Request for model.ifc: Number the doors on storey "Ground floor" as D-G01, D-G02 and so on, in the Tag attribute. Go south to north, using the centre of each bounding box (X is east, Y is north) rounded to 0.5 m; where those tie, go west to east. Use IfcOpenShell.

First a look at what the model holds.

```python
import ifcopenshell
import ifcopenshell.util.element
import ifcopenshell.util.placement

model = ifcopenshell.open("model.ifc")
print(model.schema)
storey = next(s for s in model.by_type("IfcBuildingStorey") if s.Name == "Ground floor")
doors = [e for e in ifcopenshell.util.element.get_decomposition(storey) if e.is_a("IfcDoor")]
for e in sorted(doors, key=lambda e: e.id()):
    origin = ifcopenshell.util.placement.get_local_placement(e.ObjectPlacement)[:3, 3]
    print(e.id(), e.Tag, e.Name, origin.round(2) + 0.0, sep=" | ")
```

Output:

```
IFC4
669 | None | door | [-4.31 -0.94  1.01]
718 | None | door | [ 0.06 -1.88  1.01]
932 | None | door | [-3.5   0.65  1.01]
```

```python
import ifcopenshell
import ifcopenshell.geom
import ifcopenshell.util.element
import ifcopenshell.util.shape

model = ifcopenshell.open("model.ifc")
settings = ifcopenshell.geom.settings()
settings.set("use-world-coords", True)


def centre(element):
    shape = ifcopenshell.geom.create_shape(settings, element)
    return ifcopenshell.util.shape.get_bbox_centroid(shape.geometry)


storey = next(s for s in model.by_type("IfcBuildingStorey") if s.Name == "Ground floor")
doors = [e for e in ifcopenshell.util.element.get_decomposition(storey) if e.is_a("IfcDoor")]

# Insertion points can sit at a corner or the storey origin, so sort by the geometry (in metres).
centres = {e: centre(e) for e in doors}
doors.sort(key=lambda e: (round(centres[e][1] / 0.5), centres[e][0]))

for i, e in enumerate(doors, start=1):
    number = f"D-G{i:02d}"
    e.Tag = number
    print(e.id(), number)

model.write("model_edited.ifc")
```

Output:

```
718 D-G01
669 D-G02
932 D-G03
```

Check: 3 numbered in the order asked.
